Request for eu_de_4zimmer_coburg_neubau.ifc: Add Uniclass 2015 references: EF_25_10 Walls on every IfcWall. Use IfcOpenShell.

First a look at what the model holds.

```python
import ifcopenshell

model = ifcopenshell.open("eu_de_4zimmer_coburg_neubau.ifc")
print(model.schema)
print("classifications:", [c.Name for c in model.by_type("IfcClassification")])
for ifc_class in ("IfcDoor", "IfcRoof", "IfcStair", "IfcWall", "IfcWindow"):
    print(ifc_class, len(model.by_type(ifc_class)))
```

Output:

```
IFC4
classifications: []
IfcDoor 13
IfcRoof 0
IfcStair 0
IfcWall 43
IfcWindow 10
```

```python
import ifcopenshell
import ifcopenshell.api.classification

model = ifcopenshell.open("eu_de_4zimmer_coburg_neubau.ifc")

system = ifcopenshell.api.classification.add_classification(model, classification="Uniclass 2015")

codes = {
    "IfcWall": ("EF_25_10", "Walls"),
}
for ifc_class, (code, name) in codes.items():
    products = model.by_type(ifc_class)
    ifcopenshell.api.classification.add_reference(
        model, products=products, classification=system, identification=code, name=name
    )
    print(code, len(products))

model.write("eu_de_4zimmer_coburg_neubau-out.ifc")
```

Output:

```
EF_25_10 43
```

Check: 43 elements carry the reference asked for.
